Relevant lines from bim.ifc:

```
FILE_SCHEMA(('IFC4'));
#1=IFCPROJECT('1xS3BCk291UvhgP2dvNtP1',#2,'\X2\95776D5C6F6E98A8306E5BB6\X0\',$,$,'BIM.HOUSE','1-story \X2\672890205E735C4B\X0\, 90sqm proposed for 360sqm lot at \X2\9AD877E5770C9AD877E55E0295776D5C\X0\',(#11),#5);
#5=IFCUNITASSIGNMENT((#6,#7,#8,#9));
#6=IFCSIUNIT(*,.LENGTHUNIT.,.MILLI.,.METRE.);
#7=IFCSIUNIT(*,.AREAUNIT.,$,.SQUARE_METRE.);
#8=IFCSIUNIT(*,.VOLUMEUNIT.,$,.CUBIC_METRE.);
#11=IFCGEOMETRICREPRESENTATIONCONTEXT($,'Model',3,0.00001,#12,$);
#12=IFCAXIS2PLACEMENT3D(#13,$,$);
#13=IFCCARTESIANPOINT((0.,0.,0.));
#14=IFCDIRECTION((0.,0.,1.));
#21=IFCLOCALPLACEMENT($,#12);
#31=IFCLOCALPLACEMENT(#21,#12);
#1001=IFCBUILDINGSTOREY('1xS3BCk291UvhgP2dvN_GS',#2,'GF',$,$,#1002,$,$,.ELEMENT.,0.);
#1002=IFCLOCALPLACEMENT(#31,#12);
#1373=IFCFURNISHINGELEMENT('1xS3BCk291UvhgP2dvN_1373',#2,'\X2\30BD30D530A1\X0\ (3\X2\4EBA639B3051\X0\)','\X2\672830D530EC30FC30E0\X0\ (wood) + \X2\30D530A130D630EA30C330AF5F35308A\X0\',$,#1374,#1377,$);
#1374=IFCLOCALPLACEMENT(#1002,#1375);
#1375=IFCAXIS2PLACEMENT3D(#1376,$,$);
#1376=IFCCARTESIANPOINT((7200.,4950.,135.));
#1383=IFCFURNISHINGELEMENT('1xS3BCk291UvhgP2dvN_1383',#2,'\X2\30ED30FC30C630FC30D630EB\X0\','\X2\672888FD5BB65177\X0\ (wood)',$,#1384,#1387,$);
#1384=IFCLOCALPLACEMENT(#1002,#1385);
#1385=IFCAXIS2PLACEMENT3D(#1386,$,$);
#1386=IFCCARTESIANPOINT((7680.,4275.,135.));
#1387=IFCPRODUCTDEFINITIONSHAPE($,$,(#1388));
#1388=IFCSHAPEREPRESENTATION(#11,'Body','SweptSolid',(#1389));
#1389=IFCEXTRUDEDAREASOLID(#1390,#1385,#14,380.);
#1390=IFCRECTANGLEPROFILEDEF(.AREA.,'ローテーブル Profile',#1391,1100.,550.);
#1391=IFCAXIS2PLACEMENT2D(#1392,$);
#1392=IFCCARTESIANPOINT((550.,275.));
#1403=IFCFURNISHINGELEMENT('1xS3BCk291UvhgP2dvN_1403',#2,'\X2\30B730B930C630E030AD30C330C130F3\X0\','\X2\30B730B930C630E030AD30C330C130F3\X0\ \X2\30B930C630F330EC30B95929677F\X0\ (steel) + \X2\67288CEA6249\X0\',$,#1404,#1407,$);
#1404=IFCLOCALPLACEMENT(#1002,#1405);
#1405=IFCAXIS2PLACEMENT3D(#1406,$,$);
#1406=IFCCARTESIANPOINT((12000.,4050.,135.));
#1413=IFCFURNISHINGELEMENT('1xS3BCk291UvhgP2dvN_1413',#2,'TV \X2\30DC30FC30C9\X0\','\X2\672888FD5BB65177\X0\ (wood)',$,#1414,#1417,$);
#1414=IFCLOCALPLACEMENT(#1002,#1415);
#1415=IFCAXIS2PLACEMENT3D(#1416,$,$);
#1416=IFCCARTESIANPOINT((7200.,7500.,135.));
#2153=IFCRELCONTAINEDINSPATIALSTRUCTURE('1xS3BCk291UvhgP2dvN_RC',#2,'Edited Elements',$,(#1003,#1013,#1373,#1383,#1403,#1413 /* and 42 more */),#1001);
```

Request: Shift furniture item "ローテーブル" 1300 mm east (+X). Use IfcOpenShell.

```python
import ifcopenshell
import ifcopenshell.api.geometry
import ifcopenshell.util.placement
import ifcopenshell.util.unit

model = ifcopenshell.open("bim.ifc")
unit_scale = ifcopenshell.util.unit.calculate_unit_scale(model)

item = model.by_id(1383)
matrix = ifcopenshell.util.placement.get_local_placement(item.ObjectPlacement)
matrix[0, 3] += 1.3 / unit_scale
ifcopenshell.api.geometry.edit_object_placement(model, product=item, matrix=matrix, is_si=False)

print(ifcopenshell.util.placement.get_local_placement(item.ObjectPlacement).round(3) + 0.0)

model.write("bim_edited.ifc")
```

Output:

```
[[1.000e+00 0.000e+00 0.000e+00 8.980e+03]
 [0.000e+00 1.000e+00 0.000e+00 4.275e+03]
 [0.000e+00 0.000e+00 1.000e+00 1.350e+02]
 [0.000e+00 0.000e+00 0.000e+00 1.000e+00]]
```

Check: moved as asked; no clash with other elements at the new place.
